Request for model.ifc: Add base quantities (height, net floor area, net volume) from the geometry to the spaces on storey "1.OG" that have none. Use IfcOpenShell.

First a look at what the model holds.

```python
import ifcopenshell
import ifcopenshell.util.element
import ifcopenshell.util.unit

model = ifcopenshell.open("model.ifc")
print(model.schema)
for unit_type in ("LENGTHUNIT", "AREAUNIT", "VOLUMEUNIT"):
    print(unit_type, ifcopenshell.util.unit.calculate_unit_scale(model, unit_type))
storey = next(s for s in model.by_type("IfcBuildingStorey") if s.Name == "1.OG")
spaces = [e for e in ifcopenshell.util.element.get_decomposition(storey) if e.is_a("IfcSpace")]
for e in sorted(spaces, key=lambda e: e.id()):
    print(e.id(), e.is_a(), e.Name, list(ifcopenshell.util.element.get_psets(e, qtos_only=True)), sep=" | ")
```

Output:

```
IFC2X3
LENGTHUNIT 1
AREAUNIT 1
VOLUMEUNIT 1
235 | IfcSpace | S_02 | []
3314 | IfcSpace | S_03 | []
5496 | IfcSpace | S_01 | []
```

```python
import ifcopenshell
import ifcopenshell.api.pset
import ifcopenshell.geom
import ifcopenshell.util.element
import ifcopenshell.util.shape
import ifcopenshell.util.unit

model = ifcopenshell.open("model.ifc")
unit_scale = ifcopenshell.util.unit.calculate_unit_scale(model)
area_scale = ifcopenshell.util.unit.calculate_unit_scale(model, "AREAUNIT")
volume_scale = ifcopenshell.util.unit.calculate_unit_scale(model, "VOLUMEUNIT")
settings = ifcopenshell.geom.settings()

storey = next(s for s in model.by_type("IfcBuildingStorey") if s.Name == "1.OG")
spaces = [e for e in ifcopenshell.util.element.get_decomposition(storey) if e.is_a("IfcSpace")]

for e in sorted(spaces, key=lambda e: e.id()):
    if ifcopenshell.util.element.get_psets(e, qtos_only=True, should_inherit=False):
        continue
    # Geometry comes back in metres, in the element's own axes.
    shape = ifcopenshell.geom.create_shape(settings, e)
    values = {
        "Height": ifcopenshell.util.shape.get_z(shape.geometry) / unit_scale,
        "NetFloorArea": ifcopenshell.util.shape.get_footprint_area(shape.geometry) / area_scale,
        "NetVolume": ifcopenshell.util.shape.get_volume(shape.geometry) / volume_scale,
    }
    qto = ifcopenshell.api.pset.add_qto(model, product=e, name="BaseQuantities")
    ifcopenshell.api.pset.edit_qto(model, qto=qto, properties=values)
    print(e.id(), {k: round(v, 3) for k, v in values.items()})

model.write("model-out.ifc")
```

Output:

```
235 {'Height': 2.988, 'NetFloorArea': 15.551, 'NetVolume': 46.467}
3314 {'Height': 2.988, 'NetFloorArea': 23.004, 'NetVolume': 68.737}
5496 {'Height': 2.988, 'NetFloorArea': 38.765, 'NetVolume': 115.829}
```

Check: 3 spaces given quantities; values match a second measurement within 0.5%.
